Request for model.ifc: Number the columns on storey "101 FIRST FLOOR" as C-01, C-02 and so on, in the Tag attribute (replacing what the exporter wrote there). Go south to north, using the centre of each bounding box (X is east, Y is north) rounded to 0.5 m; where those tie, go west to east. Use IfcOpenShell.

First a look at what the model holds.

```python
import ifcopenshell
import ifcopenshell.util.element
import ifcopenshell.util.placement

model = ifcopenshell.open("model.ifc")
print(model.schema)
storey = next(s for s in model.by_type("IfcBuildingStorey") if s.Name == "101 FIRST FLOOR")
columns = [e for e in ifcopenshell.util.element.get_decomposition(storey) if e.is_a("IfcColumn")]
for e in sorted(columns, key=lambda e: e.id()):
    origin = ifcopenshell.util.placement.get_local_placement(e.ObjectPlacement)[:3, 3]
    print(e.id(), e.Tag, e.Name, origin.round(2) + 0.0, sep=" | ")
```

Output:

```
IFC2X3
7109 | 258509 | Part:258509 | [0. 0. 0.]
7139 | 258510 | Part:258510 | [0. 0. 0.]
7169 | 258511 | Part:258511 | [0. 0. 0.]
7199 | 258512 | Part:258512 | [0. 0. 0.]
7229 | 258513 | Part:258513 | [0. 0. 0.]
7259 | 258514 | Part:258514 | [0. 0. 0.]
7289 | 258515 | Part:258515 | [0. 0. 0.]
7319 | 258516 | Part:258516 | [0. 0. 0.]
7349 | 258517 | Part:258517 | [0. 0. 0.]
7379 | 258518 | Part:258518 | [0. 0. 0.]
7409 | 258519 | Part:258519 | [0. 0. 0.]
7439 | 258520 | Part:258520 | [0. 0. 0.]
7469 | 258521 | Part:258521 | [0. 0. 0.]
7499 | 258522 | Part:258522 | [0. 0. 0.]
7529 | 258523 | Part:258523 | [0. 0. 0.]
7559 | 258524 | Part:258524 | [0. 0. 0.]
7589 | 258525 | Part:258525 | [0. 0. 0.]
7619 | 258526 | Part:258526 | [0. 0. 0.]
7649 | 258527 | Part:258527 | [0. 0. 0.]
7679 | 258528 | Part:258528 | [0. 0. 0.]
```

```python
import ifcopenshell
import ifcopenshell.geom
import ifcopenshell.util.element
import ifcopenshell.util.shape

model = ifcopenshell.open("model.ifc")
settings = ifcopenshell.geom.settings()
settings.set("use-world-coords", True)


def centre(element):
    shape = ifcopenshell.geom.create_shape(settings, element)
    return ifcopenshell.util.shape.get_bbox_centroid(shape.geometry)


storey = next(s for s in model.by_type("IfcBuildingStorey") if s.Name == "101 FIRST FLOOR")
columns = [e for e in ifcopenshell.util.element.get_decomposition(storey) if e.is_a("IfcColumn")]

# Insertion points can sit at a corner or the storey origin, so sort by the geometry (in metres).
centres = {e: centre(e) for e in columns}
columns.sort(key=lambda e: (round(centres[e][1] / 0.5), centres[e][0]))

for i, e in enumerate(columns, start=1):
    number = f"C-{i:02d}"
    e.Tag = number
    print(e.id(), number)

model.write("model_rev.ifc")
```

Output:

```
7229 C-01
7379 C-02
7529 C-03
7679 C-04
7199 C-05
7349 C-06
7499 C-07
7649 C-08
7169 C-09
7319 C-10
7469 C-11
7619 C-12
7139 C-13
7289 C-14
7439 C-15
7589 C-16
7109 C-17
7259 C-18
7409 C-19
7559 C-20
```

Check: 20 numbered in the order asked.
